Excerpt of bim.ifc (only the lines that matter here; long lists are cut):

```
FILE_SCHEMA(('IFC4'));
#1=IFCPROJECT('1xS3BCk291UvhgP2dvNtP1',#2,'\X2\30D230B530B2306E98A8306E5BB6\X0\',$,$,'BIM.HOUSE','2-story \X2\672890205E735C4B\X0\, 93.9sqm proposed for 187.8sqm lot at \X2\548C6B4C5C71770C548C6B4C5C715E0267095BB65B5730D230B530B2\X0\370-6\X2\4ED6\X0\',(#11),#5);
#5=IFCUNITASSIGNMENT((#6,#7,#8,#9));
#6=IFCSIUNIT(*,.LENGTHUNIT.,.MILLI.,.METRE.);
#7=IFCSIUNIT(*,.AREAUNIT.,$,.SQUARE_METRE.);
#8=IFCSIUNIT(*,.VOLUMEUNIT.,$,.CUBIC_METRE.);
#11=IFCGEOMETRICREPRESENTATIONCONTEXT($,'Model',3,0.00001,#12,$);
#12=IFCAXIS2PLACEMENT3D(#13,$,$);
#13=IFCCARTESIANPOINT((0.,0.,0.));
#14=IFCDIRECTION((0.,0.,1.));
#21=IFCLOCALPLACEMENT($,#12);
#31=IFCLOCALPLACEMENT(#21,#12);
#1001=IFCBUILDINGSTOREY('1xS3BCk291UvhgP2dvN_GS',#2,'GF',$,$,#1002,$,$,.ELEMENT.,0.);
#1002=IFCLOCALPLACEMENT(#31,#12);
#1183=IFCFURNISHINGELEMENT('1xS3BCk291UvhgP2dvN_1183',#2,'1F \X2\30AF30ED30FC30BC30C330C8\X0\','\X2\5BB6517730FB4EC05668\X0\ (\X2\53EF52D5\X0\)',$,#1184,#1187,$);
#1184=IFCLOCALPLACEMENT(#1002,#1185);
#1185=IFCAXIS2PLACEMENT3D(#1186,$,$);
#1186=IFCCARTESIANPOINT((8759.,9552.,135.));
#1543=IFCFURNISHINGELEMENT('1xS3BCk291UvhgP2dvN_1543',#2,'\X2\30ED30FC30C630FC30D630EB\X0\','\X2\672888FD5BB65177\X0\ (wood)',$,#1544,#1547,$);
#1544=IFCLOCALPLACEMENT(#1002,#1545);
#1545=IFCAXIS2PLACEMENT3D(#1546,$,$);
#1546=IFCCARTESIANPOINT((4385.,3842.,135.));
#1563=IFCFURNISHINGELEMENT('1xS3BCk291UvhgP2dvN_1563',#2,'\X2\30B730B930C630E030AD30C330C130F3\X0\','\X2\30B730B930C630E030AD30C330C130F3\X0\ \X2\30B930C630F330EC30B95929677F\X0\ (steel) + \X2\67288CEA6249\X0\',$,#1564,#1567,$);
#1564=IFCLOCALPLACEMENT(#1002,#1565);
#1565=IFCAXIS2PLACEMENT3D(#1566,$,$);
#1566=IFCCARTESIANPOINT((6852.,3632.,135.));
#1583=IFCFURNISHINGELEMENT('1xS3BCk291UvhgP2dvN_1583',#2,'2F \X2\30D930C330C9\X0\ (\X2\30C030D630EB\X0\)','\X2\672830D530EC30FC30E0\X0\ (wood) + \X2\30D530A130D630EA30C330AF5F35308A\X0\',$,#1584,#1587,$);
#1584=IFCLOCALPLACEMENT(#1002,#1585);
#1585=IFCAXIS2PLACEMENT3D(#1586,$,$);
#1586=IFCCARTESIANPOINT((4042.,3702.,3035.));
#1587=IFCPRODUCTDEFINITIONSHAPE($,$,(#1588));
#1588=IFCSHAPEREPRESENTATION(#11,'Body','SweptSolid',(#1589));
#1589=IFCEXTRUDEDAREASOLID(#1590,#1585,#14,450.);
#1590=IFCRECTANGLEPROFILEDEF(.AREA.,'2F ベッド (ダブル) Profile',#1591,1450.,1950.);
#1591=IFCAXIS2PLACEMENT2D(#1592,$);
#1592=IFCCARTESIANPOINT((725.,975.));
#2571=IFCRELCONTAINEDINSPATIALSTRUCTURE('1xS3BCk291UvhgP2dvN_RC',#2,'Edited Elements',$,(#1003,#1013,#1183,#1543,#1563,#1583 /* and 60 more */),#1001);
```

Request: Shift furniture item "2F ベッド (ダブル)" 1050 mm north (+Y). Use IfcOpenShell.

```python
import ifcopenshell
import ifcopenshell.api.geometry
import ifcopenshell.util.placement
import ifcopenshell.util.unit

model = ifcopenshell.open("bim.ifc")
unit_scale = ifcopenshell.util.unit.calculate_unit_scale(model)

item = model.by_guid("1xS3BCk291UvhgP2dvN_1583")
matrix = ifcopenshell.util.placement.get_local_placement(item.ObjectPlacement)
matrix[1, 3] += 1.05 / unit_scale
ifcopenshell.api.geometry.edit_object_placement(model, product=item, matrix=matrix, is_si=False)

print(ifcopenshell.util.placement.get_local_placement(item.ObjectPlacement).round(3) + 0.0)

model.write("bim-out.ifc")
```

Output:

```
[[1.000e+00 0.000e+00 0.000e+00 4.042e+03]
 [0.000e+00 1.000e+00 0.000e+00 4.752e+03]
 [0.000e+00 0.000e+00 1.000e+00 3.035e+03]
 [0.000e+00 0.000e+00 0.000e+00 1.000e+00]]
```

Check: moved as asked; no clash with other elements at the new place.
